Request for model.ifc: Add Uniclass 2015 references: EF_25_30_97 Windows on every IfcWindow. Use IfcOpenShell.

First a look at what the model holds.

```python
import ifcopenshell

model = ifcopenshell.open("model.ifc")
print(model.schema)
print("classifications:", [c.Name for c in model.by_type("IfcClassification")])
for ifc_class in ("IfcDoor", "IfcRoof", "IfcStair", "IfcWall", "IfcWindow"):
    print(ifc_class, len(model.by_type(ifc_class)))
```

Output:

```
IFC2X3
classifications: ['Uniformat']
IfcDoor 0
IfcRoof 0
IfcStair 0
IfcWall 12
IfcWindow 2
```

```python
import ifcopenshell
import ifcopenshell.api.classification

model = ifcopenshell.open("model.ifc")

# IFC2X3 requires Source and Edition and has no link from the project to the system.
system = model.create_entity("IfcClassification", Source="NBS", Edition="2015", Name="Uniclass 2015")

codes = {
    "IfcWindow": ("EF_25_30_97", "Windows"),
}
for ifc_class, (code, name) in codes.items():
    products = model.by_type(ifc_class)
    ifcopenshell.api.classification.add_reference(
        model, products=products, classification=system, identification=code, name=name
    )
    print(code, len(products))

model.write("model_edited.ifc")
```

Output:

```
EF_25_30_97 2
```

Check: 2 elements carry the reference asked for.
